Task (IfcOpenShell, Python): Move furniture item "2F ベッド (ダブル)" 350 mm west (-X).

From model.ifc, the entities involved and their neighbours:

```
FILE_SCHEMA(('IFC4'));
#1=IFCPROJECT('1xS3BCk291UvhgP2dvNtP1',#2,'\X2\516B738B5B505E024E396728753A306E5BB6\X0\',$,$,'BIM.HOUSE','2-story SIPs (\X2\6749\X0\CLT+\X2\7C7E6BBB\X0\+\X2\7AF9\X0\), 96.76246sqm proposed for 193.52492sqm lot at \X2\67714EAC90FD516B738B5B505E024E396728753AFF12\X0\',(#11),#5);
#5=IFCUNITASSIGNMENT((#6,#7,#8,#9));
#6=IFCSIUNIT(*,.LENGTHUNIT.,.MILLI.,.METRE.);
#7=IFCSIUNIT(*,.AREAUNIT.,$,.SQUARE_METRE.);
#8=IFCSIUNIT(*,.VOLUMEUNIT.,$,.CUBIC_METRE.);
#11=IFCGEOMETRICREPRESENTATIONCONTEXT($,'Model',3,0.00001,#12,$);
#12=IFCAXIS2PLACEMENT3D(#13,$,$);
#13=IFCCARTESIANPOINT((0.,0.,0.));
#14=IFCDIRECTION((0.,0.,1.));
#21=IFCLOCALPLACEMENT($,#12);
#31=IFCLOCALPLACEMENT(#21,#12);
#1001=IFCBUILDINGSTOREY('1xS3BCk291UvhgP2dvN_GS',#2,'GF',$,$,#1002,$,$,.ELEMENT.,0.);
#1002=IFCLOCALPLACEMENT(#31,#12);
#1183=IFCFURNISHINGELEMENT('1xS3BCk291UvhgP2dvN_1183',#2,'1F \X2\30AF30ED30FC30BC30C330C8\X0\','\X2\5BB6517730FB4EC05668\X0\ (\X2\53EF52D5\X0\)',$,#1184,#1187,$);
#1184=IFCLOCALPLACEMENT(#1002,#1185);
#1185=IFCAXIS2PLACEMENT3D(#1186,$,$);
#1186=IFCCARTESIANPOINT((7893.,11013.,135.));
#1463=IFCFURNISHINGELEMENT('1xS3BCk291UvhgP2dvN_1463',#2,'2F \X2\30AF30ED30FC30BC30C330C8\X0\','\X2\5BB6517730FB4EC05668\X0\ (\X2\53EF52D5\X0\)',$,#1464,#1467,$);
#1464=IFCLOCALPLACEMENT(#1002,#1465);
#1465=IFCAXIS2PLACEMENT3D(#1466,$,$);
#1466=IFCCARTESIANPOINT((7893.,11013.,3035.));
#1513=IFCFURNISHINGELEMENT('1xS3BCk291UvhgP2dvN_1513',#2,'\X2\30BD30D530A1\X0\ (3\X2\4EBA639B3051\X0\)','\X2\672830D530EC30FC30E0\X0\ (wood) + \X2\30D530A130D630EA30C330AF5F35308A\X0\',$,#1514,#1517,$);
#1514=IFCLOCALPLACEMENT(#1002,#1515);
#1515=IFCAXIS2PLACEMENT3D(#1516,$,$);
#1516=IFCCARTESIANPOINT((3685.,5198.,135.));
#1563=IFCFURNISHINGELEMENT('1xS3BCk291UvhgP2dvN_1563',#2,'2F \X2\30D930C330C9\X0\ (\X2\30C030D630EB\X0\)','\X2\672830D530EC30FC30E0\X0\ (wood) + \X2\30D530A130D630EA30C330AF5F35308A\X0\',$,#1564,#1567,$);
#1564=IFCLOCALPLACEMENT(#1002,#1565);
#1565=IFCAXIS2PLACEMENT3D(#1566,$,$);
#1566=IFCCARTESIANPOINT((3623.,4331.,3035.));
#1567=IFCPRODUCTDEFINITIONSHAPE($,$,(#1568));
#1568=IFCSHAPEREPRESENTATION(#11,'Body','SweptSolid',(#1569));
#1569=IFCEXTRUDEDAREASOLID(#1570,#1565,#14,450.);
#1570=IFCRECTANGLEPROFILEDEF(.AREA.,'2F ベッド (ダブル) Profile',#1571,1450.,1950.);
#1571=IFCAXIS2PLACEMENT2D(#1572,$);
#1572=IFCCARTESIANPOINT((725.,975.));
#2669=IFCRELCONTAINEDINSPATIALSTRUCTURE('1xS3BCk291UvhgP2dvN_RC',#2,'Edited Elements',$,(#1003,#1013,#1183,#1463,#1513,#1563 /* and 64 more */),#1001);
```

```python
import ifcopenshell
import ifcopenshell.api.geometry
import ifcopenshell.util.placement

model = ifcopenshell.open("model.ifc")

item = model.by_id(1563)
matrix = ifcopenshell.util.placement.get_local_placement(item.ObjectPlacement)
matrix[0, 3] -= 350.0
ifcopenshell.api.geometry.edit_object_placement(model, product=item, matrix=matrix, is_si=False)

print(ifcopenshell.util.placement.get_local_placement(item.ObjectPlacement).round(3) + 0.0)

model.write("model_edited.ifc")
```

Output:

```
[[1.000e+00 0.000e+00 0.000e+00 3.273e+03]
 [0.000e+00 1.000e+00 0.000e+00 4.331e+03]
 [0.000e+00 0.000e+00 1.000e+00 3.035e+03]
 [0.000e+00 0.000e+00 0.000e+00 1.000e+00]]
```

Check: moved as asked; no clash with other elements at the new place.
